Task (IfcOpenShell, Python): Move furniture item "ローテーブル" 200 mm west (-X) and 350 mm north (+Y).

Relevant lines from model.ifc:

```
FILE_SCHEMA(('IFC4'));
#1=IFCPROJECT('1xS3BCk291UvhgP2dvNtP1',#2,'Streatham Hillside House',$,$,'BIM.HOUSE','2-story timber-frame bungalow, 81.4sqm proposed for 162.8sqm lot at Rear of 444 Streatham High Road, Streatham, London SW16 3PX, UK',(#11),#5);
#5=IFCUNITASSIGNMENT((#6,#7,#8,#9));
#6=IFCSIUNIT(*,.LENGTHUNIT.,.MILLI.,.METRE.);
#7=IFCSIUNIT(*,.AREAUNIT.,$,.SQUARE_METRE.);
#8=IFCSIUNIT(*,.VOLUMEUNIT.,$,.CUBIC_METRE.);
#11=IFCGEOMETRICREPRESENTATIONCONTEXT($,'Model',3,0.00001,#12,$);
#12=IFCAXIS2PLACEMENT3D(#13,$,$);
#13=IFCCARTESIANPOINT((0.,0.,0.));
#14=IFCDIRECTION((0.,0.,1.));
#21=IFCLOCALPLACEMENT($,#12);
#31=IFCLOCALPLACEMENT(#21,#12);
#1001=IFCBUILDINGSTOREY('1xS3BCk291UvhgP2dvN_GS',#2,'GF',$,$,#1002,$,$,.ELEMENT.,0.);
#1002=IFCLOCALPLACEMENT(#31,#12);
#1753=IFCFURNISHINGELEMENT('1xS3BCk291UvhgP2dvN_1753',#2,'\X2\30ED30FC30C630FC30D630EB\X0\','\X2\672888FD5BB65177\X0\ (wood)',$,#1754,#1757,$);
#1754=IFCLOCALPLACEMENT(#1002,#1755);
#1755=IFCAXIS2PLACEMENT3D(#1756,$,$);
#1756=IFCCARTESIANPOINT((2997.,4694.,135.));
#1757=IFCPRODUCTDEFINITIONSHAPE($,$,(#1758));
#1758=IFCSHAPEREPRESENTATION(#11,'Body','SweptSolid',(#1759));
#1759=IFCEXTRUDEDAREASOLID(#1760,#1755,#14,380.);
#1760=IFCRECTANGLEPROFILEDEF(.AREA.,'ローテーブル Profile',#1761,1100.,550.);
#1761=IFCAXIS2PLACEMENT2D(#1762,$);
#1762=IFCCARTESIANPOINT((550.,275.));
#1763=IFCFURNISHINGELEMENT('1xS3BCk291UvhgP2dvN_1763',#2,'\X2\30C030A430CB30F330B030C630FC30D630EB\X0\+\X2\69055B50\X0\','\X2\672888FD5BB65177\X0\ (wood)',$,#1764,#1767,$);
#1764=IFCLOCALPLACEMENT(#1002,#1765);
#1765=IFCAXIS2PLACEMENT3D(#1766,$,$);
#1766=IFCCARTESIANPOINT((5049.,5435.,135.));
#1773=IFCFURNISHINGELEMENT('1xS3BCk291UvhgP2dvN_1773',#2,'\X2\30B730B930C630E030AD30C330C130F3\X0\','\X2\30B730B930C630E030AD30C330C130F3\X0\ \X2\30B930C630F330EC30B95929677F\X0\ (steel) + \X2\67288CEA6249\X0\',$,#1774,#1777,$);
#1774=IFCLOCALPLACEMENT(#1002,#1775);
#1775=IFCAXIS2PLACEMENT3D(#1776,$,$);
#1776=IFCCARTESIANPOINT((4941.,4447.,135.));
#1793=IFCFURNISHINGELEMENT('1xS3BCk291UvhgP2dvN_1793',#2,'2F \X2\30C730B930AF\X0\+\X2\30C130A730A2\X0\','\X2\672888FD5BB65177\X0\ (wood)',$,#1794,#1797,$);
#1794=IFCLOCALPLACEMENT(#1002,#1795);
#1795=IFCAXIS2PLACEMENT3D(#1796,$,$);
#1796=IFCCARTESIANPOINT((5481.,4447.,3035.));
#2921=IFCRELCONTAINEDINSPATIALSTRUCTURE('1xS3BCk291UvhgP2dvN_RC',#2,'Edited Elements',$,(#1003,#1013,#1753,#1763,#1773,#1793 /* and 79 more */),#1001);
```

```python
import ifcopenshell
import ifcopenshell.api.geometry
import ifcopenshell.util.placement

model = ifcopenshell.open("model.ifc")

item = model.by_guid("1xS3BCk291UvhgP2dvN_1753")
matrix = ifcopenshell.util.placement.get_local_placement(item.ObjectPlacement)
matrix[0, 3] -= 200.0
matrix[1, 3] += 350.0
ifcopenshell.api.geometry.edit_object_placement(model, product=item, matrix=matrix, is_si=False)

print(ifcopenshell.util.placement.get_local_placement(item.ObjectPlacement).round(3) + 0.0)

model.write("model_edited.ifc")
```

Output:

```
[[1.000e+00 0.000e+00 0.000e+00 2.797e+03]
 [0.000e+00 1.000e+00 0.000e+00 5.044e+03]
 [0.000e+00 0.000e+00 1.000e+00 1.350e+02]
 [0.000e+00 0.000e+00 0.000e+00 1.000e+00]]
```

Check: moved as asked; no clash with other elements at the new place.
